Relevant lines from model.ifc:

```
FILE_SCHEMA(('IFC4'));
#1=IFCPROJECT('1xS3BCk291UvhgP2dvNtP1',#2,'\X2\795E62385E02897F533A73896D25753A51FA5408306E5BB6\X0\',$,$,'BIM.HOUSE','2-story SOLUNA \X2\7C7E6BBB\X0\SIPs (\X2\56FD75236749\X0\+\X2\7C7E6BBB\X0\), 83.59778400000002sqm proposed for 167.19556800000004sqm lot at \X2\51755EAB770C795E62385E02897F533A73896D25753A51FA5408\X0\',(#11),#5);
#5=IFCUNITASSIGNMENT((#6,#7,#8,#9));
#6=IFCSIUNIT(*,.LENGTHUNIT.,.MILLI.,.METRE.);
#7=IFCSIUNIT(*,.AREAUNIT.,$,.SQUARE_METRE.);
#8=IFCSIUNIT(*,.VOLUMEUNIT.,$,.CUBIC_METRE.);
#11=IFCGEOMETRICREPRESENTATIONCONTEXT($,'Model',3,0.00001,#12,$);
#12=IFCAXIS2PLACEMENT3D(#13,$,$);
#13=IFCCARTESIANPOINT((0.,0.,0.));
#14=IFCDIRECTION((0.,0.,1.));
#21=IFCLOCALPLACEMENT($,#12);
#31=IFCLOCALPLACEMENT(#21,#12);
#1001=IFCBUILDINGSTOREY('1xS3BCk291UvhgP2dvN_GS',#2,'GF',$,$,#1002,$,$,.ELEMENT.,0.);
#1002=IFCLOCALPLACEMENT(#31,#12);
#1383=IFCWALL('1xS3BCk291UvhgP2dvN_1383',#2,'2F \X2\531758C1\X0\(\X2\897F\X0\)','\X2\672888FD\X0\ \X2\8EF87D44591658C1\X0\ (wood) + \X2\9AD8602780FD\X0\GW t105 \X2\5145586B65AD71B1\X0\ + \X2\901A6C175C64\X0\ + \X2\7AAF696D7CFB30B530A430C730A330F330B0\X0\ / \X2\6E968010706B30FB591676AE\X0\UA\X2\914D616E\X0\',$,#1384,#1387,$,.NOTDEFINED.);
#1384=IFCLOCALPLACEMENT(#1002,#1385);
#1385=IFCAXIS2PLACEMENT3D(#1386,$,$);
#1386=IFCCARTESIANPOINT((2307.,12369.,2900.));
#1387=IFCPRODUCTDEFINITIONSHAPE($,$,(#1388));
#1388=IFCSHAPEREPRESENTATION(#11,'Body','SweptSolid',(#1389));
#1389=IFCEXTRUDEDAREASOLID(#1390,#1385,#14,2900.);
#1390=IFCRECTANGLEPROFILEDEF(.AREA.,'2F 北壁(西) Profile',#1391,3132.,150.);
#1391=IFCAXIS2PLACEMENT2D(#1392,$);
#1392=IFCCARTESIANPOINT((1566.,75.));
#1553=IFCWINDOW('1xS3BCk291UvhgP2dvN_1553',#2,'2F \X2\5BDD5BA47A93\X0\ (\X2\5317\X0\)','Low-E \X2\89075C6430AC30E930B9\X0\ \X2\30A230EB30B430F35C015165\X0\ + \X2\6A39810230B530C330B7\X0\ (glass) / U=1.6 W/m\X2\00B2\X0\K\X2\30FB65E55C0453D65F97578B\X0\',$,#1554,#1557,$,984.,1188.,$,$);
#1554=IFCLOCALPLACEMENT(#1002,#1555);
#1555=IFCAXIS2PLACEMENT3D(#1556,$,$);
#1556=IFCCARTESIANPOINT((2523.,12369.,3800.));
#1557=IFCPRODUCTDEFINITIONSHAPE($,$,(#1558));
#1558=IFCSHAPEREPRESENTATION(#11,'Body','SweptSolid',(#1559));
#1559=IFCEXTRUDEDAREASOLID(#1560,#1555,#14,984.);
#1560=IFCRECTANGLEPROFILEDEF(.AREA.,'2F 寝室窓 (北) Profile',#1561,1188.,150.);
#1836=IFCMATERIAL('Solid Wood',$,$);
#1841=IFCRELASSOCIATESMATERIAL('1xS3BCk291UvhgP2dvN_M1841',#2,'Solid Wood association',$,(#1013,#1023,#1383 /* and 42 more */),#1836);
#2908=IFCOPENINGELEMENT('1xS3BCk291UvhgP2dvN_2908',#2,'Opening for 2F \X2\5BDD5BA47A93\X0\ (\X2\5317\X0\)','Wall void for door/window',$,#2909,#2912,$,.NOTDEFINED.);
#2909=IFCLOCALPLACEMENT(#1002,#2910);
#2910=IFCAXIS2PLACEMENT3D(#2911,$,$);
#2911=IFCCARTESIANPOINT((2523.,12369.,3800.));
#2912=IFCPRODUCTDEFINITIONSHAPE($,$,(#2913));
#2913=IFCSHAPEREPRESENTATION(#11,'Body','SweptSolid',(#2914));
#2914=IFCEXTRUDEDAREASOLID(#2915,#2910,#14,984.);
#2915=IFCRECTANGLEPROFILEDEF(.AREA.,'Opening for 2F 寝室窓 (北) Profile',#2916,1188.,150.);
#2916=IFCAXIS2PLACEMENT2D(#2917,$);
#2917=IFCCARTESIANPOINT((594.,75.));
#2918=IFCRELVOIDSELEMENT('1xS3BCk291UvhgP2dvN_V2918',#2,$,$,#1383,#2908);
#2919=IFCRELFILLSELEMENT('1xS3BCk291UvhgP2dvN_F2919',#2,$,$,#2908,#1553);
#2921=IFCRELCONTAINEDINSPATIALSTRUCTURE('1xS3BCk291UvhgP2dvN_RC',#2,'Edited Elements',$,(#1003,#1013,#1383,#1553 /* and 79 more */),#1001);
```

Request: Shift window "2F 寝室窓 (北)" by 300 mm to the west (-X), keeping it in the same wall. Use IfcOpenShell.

```python
import ifcopenshell
import ifcopenshell.api.geometry
import ifcopenshell.util.placement
import ifcopenshell.util.unit

model = ifcopenshell.open("model.ifc")
unit_scale = ifcopenshell.util.unit.calculate_unit_scale(model)

window = model.by_guid("1xS3BCk291UvhgP2dvN_1553")
opening = window.FillsVoids[0].RelatingOpeningElement
wall = opening.VoidsElements[0].RelatingBuildingElement

wall_matrix = ifcopenshell.util.placement.get_local_placement(wall.ObjectPlacement)
shift = wall_matrix[:3, 0] * -0.3 / unit_scale
before = ifcopenshell.util.placement.get_local_placement(window.ObjectPlacement)[:3, 3].copy()

# The window is not placed relative to its opening, so move both.
for product in (opening, window):
    matrix = ifcopenshell.util.placement.get_local_placement(product.ObjectPlacement)
    matrix[:3, 3] += shift
    ifcopenshell.api.geometry.edit_object_placement(model, product=product, matrix=matrix, is_si=False)

after = ifcopenshell.util.placement.get_local_placement(window.ObjectPlacement)[:3, 3]
print("window moved by", (after - before).round(3) + 0.0)

model.write("model_edited.ifc")
```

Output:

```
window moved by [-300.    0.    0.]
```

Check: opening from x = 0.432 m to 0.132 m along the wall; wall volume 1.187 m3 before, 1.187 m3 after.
